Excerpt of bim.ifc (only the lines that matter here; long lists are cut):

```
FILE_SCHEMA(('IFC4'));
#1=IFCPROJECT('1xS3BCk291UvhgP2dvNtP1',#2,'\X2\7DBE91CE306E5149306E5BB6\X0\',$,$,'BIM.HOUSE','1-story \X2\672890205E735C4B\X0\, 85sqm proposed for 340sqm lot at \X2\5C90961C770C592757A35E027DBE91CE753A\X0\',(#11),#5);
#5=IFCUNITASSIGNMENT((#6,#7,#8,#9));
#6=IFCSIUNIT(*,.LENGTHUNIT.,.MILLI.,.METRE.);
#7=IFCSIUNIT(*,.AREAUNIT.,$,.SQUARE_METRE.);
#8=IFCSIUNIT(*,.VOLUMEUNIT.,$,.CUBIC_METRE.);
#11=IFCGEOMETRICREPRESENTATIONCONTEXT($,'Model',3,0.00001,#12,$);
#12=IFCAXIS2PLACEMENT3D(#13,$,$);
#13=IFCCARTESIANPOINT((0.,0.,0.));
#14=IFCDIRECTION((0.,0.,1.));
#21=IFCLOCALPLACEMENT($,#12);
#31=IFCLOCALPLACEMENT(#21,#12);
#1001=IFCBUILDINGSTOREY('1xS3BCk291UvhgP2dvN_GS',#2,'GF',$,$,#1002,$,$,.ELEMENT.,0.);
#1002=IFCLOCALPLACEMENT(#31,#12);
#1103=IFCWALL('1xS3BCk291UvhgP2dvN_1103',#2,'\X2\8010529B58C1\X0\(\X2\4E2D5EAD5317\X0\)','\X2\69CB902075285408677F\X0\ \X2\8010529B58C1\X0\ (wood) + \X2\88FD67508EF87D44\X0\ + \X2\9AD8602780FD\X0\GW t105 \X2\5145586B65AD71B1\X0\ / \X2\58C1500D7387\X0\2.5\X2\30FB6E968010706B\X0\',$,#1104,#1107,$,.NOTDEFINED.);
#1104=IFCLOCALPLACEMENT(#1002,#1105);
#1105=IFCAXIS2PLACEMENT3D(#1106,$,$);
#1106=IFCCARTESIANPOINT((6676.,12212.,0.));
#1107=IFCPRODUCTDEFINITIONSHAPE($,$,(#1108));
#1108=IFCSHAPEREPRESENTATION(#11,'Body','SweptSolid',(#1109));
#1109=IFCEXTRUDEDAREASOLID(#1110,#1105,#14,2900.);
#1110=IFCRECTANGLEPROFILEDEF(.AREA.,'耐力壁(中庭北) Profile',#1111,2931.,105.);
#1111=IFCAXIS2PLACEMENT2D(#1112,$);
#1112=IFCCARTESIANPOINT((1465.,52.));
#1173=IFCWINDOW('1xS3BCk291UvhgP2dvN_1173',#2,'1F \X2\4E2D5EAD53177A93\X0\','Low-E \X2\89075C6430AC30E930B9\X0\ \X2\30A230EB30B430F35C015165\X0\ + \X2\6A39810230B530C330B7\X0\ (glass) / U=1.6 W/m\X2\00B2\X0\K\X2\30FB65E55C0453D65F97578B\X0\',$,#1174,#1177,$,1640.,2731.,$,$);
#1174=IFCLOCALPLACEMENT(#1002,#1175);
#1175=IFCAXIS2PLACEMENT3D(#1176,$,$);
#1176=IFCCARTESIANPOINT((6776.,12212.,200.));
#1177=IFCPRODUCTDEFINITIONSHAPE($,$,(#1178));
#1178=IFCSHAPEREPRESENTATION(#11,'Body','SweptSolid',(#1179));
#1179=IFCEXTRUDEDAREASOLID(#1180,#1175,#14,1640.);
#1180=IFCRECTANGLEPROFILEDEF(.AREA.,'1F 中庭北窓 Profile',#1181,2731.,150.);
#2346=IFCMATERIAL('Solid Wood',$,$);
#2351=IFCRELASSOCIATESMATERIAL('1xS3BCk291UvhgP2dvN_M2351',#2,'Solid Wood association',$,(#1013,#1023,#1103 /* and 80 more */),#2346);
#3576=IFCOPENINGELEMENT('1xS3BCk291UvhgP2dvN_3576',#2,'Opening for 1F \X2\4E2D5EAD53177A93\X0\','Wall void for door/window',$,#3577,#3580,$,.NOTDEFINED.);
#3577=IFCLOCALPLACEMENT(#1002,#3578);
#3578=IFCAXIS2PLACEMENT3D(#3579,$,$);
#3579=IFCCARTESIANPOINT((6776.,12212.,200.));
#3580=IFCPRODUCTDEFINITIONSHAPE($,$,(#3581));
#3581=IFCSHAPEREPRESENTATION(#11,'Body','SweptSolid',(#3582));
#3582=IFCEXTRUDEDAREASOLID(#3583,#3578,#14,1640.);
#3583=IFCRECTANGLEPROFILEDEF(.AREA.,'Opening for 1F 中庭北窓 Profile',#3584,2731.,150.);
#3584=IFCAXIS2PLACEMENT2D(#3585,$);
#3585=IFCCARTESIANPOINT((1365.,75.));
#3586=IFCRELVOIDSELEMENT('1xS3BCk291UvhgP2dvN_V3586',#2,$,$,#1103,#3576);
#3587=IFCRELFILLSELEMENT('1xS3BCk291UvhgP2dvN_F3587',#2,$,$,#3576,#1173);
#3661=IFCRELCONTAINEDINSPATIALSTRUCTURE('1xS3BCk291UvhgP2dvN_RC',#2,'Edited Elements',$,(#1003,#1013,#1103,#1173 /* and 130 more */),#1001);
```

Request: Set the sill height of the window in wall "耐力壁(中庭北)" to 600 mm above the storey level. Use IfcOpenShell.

```python
import numpy as np
import ifcopenshell
import ifcopenshell.api.geometry
import ifcopenshell.geom
import ifcopenshell.util.element
import ifcopenshell.util.placement
import ifcopenshell.util.shape
import ifcopenshell.util.unit

model = ifcopenshell.open("bim.ifc")
unit_scale = ifcopenshell.util.unit.calculate_unit_scale(model)

window = model.by_guid("1xS3BCk291UvhgP2dvN_1173")
opening = window.FillsVoids[0].RelatingOpeningElement
storey = ifcopenshell.util.element.get_container(window, ifc_class="IfcBuildingStorey")
level = ifcopenshell.util.placement.get_local_placement(storey.ObjectPlacement)[2, 3]

# The opening's origin need not be at the sill, so measure its lowest point.
shape = ifcopenshell.geom.create_shape(ifcopenshell.geom.settings(), opening)
bottom = ifcopenshell.util.shape.get_shape_bottom_elevation(shape, shape.geometry) / unit_scale
dz = level + 0.6 / unit_scale - bottom

shift = np.array([0.0, 0.0, dz])
# The window is not placed relative to its opening, so move both.
for product in (opening, window):
    matrix = ifcopenshell.util.placement.get_local_placement(product.ObjectPlacement)
    matrix[:3, 3] += shift
    ifcopenshell.api.geometry.edit_object_placement(model, product=product, matrix=matrix, is_si=False)

print(f"moved by {dz * unit_scale:+.3f} m")

model.write("bim_rev.ifc")
```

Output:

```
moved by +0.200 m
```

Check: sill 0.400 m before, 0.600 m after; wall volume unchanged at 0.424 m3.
